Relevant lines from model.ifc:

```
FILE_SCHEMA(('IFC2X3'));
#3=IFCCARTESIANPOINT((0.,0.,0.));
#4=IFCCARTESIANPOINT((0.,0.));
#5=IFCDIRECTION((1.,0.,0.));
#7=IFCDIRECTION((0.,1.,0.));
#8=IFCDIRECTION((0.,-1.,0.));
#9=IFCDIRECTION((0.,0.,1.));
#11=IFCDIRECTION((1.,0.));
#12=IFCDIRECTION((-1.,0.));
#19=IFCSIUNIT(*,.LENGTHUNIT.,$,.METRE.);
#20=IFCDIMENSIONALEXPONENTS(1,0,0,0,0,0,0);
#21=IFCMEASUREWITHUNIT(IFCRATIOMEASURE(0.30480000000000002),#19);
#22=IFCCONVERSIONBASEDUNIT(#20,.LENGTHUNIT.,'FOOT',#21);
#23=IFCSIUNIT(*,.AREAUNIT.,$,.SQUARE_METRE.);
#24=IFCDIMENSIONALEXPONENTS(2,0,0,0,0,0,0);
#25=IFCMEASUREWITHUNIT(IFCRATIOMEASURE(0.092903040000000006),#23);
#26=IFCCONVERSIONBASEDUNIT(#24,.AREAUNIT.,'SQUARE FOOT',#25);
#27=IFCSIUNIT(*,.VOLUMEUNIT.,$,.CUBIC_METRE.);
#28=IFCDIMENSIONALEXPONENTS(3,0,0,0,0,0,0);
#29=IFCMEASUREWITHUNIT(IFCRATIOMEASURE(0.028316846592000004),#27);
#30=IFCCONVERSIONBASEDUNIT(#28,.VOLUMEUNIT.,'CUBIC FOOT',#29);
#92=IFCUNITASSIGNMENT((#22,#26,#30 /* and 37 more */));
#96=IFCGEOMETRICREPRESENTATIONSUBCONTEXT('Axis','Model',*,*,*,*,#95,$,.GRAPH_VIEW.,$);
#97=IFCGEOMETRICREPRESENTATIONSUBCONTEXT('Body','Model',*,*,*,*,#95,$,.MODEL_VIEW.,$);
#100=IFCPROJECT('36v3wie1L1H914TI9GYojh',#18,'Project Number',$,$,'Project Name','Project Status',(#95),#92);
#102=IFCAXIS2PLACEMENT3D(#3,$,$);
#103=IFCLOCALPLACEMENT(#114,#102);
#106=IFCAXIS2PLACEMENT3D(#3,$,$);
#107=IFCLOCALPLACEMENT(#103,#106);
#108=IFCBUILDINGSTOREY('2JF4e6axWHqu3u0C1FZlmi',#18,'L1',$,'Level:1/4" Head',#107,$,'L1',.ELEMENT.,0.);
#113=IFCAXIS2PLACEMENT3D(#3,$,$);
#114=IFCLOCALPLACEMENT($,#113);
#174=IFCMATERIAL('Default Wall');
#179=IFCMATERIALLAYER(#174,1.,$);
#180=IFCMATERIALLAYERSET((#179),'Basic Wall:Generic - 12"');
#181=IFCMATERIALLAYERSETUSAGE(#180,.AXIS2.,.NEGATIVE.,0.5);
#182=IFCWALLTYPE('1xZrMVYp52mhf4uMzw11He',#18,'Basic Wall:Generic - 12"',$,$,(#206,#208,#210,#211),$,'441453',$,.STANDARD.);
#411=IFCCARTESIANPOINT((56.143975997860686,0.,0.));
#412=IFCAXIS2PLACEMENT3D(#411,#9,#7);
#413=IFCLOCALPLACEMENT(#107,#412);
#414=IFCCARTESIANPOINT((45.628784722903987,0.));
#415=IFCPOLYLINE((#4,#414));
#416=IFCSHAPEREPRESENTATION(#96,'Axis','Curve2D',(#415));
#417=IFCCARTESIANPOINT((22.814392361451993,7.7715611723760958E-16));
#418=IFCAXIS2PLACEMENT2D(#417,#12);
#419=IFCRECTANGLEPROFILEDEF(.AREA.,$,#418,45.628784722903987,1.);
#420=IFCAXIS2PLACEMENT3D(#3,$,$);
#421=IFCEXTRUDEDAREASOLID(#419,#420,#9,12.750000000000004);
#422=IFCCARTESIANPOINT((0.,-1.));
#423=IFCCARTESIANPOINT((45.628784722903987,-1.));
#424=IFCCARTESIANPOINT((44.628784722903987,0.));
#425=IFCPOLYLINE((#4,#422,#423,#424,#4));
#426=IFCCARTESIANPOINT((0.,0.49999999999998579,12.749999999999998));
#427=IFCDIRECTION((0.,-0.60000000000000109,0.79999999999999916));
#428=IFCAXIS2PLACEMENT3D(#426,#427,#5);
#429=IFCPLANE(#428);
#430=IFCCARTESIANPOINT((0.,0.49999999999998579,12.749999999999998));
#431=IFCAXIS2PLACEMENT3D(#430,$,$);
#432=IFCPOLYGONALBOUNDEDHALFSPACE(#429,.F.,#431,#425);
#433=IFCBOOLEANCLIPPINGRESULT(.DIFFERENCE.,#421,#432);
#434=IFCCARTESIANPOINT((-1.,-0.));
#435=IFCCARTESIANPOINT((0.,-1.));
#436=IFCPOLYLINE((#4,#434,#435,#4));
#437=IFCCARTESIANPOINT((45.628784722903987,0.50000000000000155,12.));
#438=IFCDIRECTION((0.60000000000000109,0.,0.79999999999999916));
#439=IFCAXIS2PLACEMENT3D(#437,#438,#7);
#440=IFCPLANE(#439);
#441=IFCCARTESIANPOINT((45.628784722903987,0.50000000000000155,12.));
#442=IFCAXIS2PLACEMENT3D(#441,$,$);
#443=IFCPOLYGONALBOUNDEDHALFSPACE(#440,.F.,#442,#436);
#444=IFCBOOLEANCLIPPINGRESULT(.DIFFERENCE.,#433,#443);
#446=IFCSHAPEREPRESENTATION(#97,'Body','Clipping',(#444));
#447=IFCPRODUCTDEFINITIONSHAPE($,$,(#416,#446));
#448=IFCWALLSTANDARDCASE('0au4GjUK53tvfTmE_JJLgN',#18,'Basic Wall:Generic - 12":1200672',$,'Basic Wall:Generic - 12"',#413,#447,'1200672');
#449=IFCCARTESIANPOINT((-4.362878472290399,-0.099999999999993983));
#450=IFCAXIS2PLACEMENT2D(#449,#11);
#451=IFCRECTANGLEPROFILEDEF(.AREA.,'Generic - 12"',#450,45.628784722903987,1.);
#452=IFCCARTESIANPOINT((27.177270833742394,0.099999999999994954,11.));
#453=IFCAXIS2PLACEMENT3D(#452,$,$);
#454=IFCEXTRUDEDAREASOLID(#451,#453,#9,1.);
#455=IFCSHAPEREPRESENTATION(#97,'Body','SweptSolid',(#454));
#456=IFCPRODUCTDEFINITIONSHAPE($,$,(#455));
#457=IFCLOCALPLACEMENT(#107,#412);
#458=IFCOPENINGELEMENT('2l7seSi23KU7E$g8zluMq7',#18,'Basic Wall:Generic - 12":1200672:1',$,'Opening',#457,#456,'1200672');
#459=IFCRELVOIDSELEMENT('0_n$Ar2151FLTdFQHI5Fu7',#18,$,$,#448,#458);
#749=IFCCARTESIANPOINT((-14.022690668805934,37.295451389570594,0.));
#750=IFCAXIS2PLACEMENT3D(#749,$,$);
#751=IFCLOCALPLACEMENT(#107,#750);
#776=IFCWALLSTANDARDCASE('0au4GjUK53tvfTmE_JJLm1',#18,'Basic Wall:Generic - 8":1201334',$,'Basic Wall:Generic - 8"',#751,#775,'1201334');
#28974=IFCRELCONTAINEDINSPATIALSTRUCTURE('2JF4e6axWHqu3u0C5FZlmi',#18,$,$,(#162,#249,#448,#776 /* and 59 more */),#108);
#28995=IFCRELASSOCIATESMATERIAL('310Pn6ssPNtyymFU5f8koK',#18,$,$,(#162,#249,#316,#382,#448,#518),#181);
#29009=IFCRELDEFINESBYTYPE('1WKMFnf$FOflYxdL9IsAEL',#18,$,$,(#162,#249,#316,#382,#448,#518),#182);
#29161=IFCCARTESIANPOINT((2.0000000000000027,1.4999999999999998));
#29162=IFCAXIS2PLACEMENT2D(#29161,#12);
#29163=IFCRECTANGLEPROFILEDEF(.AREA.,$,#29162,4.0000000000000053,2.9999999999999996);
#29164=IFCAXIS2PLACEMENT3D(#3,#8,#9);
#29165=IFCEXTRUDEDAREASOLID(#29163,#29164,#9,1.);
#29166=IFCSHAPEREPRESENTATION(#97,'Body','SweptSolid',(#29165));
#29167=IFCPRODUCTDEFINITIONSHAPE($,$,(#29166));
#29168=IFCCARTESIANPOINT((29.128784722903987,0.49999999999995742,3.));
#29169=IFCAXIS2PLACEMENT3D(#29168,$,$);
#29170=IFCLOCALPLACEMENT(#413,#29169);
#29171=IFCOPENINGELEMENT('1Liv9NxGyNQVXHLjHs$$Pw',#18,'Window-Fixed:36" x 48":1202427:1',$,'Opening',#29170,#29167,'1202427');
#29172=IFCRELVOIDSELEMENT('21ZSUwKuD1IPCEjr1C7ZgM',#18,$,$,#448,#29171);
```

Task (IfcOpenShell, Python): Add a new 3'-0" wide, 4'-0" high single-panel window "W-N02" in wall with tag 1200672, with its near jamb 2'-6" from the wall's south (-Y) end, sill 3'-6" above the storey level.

```python
import numpy as np
import ifcopenshell
import ifcopenshell.api.feature
import ifcopenshell.api.geometry
import ifcopenshell.api.root
import ifcopenshell.api.spatial
import ifcopenshell.api.type
import ifcopenshell.geom
import ifcopenshell.util.element
import ifcopenshell.util.placement
import ifcopenshell.util.representation
import ifcopenshell.util.shape
import ifcopenshell.util.unit

model = ifcopenshell.open("model.ifc")
unit_scale = ifcopenshell.util.unit.calculate_unit_scale(model)
settings = ifcopenshell.geom.settings()


def volume(element):
    """Net volume in cubic metres, openings subtracted."""
    shape = ifcopenshell.geom.create_shape(settings, element)
    return ifcopenshell.util.shape.get_volume(shape.geometry)


wall = model.by_id(448)
storey = ifcopenshell.util.element.get_container(wall, ifc_class="IfcBuildingStorey")
context = ifcopenshell.util.representation.get_context(model, "Model", "Body", "MODEL_VIEW")
before = volume(wall)

width, height, from_end, sill = 0.9144, 1.2192, 0.762, 1.0668  # metres

# The wall runs along its own X axis, and the end named is its -X end.
wall_shape = ifcopenshell.geom.create_shape(settings, wall)
x, y, z = ifcopenshell.util.shape.get_vertices(wall_shape.geometry).T
start = x.min() + from_end
face, thickness = float(y.min()), float(y.max() - y.min())
wall_matrix = ifcopenshell.util.placement.get_local_placement(wall.ObjectPlacement)
level = ifcopenshell.util.placement.get_local_placement(storey.ObjectPlacement)[2, 3]


def in_wall(x, y):
    """Placement at x, y metres in the wall's axes, at sill height."""
    matrix = wall_matrix.copy()
    matrix[:, 3] = wall_matrix @ np.array([x / unit_scale, y / unit_scale, 0.0, 1.0])
    matrix[2, 3] = level + sill / unit_scale
    return matrix


# Opening: a box that overshoots both wall faces by 50 mm.
opening = ifcopenshell.api.root.create_entity(model, ifc_class="IfcOpeningElement")
box = ifcopenshell.api.geometry.add_wall_representation(
    model, context=context, length=width, height=height, thickness=thickness + 0.1
)
ifcopenshell.api.geometry.assign_representation(model, product=opening, representation=box)
ifcopenshell.api.geometry.edit_object_placement(model, product=opening, matrix=in_wall(start, face - 0.05), is_si=False)
ifcopenshell.api.feature.add_feature(model, feature=opening, element=wall)

window = ifcopenshell.api.root.create_entity(model, ifc_class="IfcWindow", name="W-N02")
window.OverallWidth, window.OverallHeight = width / unit_scale, height / unit_scale
body = ifcopenshell.api.geometry.add_window_representation(
    model,
    context=context,
    overall_width=window.OverallWidth,
    overall_height=window.OverallHeight,
    partition_type="SINGLE_PANEL",
)
ifcopenshell.api.geometry.assign_representation(model, product=window, representation=body)
ifcopenshell.api.spatial.assign_container(model, products=[window], relating_structure=storey)
fills = ifcopenshell.api.feature.add_filling(model, opening=opening, element=window)
fills.OwnerHistory = window.OwnerHistory  # required in IFC2X3

# IFC2X3 keeps the operation on the window style.
style = ifcopenshell.api.root.create_entity(model, ifc_class="IfcWindowStyle", name="W-N02")
style.OperationType, style.ConstructionType = "SINGLE_PANEL", "NOTDEFINED"
style.ParameterTakesPrecedence = style.Sizeable = False
ifcopenshell.api.type.assign_type(model, related_objects=[window], relating_type=style)

# Centre the window in the wall's thickness.
ifcopenshell.api.geometry.edit_object_placement(model, product=window, matrix=in_wall(start, face), is_si=False)
window_shape = ifcopenshell.geom.create_shape(settings, window)
depth = ifcopenshell.util.shape.get_vertices(window_shape.geometry)[:, 1]
offset = face + thickness / 2 - (depth.min() + depth.max()) / 2
ifcopenshell.api.geometry.edit_object_placement(model, product=window, matrix=in_wall(start, offset), is_si=False)

after = volume(wall)

print(f"wall volume {before:.3f} -> {after:.3f} m3")

model.write("model-out.ifc")
```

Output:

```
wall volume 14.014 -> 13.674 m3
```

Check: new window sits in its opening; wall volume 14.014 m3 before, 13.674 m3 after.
